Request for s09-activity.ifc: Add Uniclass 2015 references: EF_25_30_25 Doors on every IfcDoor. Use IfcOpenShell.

First a look at what the model holds.

```python
import ifcopenshell

model = ifcopenshell.open("s09-activity.ifc")
print(model.schema)
print("classifications:", [c.Name for c in model.by_type("IfcClassification")])
for ifc_class in ("IfcDoor", "IfcRoof", "IfcStair", "IfcWall", "IfcWindow"):
    print(ifc_class, len(model.by_type(ifc_class)))
```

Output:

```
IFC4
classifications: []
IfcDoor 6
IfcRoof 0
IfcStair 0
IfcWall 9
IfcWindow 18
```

```python
import ifcopenshell
import ifcopenshell.api.classification

model = ifcopenshell.open("s09-activity.ifc")

system = ifcopenshell.api.classification.add_classification(model, classification="Uniclass 2015")

codes = {
    "IfcDoor": ("EF_25_30_25", "Doors"),
}
for ifc_class, (code, name) in codes.items():
    products = model.by_type(ifc_class)
    ifcopenshell.api.classification.add_reference(
        model, products=products, classification=system, identification=code, name=name
    )
    print(code, len(products))

model.write("s09-activity-out.ifc")
```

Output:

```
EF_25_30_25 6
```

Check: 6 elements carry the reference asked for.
